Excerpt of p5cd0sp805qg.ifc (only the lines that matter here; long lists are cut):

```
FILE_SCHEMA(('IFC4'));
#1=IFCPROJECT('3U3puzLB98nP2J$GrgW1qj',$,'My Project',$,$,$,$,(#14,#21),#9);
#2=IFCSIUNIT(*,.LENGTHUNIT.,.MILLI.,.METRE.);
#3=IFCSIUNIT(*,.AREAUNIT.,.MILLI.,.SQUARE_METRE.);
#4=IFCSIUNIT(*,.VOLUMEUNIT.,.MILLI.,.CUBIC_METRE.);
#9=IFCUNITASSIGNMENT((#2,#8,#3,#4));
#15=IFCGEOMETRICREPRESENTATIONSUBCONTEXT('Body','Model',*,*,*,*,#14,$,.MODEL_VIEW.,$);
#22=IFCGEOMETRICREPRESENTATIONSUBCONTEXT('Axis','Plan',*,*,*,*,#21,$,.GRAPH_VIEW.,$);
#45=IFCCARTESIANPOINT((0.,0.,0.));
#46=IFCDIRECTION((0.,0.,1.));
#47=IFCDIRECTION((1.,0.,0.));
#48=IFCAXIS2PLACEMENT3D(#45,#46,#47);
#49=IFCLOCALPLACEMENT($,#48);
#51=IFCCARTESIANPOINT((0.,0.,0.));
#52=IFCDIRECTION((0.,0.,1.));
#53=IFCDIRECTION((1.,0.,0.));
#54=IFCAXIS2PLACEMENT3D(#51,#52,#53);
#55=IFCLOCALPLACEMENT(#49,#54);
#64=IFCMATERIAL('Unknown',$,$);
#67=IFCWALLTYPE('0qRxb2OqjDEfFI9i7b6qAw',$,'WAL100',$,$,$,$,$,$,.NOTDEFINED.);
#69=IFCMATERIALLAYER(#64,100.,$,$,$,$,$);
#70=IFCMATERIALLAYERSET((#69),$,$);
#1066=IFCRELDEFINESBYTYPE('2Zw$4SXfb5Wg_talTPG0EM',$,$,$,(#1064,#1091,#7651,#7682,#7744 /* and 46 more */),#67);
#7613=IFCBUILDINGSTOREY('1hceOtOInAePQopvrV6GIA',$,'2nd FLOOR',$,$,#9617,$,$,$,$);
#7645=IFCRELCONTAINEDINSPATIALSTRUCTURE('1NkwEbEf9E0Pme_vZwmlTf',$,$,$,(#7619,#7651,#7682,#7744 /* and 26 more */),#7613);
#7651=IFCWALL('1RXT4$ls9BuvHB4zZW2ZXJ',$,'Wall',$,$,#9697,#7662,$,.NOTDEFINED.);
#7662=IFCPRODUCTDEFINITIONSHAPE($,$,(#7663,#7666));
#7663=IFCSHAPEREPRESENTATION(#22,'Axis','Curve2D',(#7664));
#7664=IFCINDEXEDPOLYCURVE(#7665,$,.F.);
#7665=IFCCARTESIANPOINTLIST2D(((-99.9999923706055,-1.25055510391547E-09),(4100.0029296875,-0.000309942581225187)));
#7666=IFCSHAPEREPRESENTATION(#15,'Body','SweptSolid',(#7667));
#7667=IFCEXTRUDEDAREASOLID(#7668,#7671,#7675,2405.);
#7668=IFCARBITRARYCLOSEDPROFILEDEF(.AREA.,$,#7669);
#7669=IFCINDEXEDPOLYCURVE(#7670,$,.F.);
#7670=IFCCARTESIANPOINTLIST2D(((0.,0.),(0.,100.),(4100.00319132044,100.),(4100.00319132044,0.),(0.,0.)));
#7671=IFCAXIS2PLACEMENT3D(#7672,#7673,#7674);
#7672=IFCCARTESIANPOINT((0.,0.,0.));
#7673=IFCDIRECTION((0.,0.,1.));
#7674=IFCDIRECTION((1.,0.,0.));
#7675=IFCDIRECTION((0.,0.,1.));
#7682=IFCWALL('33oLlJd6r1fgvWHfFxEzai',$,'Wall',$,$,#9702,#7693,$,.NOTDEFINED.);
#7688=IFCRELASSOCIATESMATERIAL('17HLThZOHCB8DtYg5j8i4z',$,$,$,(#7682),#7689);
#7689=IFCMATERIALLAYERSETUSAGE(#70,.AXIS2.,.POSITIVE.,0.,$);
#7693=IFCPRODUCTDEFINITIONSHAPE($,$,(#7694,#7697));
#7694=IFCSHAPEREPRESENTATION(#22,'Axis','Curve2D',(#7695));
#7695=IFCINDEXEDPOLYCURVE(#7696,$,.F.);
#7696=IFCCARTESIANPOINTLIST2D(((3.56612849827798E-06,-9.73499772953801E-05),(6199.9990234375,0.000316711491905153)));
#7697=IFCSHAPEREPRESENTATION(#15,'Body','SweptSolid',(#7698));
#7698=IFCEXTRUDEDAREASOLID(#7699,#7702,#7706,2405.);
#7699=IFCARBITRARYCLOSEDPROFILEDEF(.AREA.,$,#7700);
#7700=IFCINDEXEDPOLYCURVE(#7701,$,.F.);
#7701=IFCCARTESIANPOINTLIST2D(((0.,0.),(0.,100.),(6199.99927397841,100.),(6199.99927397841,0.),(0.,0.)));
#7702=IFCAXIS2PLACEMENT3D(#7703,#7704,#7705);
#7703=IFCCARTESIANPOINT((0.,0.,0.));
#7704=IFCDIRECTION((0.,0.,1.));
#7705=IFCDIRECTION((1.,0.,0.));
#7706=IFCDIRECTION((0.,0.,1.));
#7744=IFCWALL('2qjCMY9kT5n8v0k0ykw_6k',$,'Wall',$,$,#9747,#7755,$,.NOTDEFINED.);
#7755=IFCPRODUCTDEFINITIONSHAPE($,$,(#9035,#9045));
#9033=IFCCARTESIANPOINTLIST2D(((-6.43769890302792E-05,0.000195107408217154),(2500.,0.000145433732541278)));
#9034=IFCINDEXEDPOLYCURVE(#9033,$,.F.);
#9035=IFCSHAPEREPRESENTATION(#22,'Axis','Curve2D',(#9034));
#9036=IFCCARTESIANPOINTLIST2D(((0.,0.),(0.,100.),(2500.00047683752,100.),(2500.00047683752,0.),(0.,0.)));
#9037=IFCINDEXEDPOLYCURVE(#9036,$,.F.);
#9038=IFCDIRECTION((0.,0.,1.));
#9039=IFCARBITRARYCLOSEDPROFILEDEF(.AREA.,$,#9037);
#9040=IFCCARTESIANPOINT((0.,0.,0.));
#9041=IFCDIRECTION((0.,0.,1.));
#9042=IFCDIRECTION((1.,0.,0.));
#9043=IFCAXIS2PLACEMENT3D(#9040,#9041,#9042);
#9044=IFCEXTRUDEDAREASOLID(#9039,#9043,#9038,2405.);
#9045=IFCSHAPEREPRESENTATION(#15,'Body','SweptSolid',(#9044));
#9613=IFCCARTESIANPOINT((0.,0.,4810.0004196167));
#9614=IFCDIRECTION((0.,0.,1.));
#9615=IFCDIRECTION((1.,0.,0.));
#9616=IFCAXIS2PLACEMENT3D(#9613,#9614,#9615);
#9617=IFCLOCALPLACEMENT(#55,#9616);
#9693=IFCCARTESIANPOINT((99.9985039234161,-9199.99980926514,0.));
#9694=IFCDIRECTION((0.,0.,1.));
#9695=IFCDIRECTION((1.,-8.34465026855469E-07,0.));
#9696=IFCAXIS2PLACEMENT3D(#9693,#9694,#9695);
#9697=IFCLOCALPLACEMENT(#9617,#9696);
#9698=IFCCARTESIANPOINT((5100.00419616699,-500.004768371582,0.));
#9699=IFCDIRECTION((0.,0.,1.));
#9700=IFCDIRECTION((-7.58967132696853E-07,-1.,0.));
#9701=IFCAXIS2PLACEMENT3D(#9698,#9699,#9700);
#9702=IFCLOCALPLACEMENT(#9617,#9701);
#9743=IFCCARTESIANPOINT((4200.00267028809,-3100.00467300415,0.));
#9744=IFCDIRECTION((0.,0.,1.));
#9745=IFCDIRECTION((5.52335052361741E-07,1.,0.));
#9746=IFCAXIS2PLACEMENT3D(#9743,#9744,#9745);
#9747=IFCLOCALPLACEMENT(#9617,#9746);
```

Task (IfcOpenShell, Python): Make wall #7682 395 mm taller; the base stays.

```python
import ifcopenshell
import ifcopenshell.geom
import ifcopenshell.util.representation
import ifcopenshell.util.shape
import ifcopenshell.util.unit

model = ifcopenshell.open("p5cd0sp805qg.ifc")
unit_scale = ifcopenshell.util.unit.calculate_unit_scale(model)
settings = ifcopenshell.geom.settings()


def volume(element):
    """Net volume in cubic metres, openings subtracted."""
    shape = ifcopenshell.geom.create_shape(settings, element)
    return ifcopenshell.util.shape.get_volume(shape.geometry)


wall = model.by_guid("33oLlJd6r1fgvWHfFxEzai")
before = volume(wall)

body = ifcopenshell.util.representation.get_representation(wall, "Model", "Body")
solid = body.Items[0]
old_height = solid.Depth
solid.Depth += 0.395 / unit_scale
after = volume(wall)

print(f"height {old_height:g} -> {solid.Depth:g}, volume {before:.3f} -> {after:.3f} m3")

model.write("p5cd0sp805qg_edited.ifc")
```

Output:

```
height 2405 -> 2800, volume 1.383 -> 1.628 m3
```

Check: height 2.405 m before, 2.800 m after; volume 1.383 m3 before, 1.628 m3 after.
